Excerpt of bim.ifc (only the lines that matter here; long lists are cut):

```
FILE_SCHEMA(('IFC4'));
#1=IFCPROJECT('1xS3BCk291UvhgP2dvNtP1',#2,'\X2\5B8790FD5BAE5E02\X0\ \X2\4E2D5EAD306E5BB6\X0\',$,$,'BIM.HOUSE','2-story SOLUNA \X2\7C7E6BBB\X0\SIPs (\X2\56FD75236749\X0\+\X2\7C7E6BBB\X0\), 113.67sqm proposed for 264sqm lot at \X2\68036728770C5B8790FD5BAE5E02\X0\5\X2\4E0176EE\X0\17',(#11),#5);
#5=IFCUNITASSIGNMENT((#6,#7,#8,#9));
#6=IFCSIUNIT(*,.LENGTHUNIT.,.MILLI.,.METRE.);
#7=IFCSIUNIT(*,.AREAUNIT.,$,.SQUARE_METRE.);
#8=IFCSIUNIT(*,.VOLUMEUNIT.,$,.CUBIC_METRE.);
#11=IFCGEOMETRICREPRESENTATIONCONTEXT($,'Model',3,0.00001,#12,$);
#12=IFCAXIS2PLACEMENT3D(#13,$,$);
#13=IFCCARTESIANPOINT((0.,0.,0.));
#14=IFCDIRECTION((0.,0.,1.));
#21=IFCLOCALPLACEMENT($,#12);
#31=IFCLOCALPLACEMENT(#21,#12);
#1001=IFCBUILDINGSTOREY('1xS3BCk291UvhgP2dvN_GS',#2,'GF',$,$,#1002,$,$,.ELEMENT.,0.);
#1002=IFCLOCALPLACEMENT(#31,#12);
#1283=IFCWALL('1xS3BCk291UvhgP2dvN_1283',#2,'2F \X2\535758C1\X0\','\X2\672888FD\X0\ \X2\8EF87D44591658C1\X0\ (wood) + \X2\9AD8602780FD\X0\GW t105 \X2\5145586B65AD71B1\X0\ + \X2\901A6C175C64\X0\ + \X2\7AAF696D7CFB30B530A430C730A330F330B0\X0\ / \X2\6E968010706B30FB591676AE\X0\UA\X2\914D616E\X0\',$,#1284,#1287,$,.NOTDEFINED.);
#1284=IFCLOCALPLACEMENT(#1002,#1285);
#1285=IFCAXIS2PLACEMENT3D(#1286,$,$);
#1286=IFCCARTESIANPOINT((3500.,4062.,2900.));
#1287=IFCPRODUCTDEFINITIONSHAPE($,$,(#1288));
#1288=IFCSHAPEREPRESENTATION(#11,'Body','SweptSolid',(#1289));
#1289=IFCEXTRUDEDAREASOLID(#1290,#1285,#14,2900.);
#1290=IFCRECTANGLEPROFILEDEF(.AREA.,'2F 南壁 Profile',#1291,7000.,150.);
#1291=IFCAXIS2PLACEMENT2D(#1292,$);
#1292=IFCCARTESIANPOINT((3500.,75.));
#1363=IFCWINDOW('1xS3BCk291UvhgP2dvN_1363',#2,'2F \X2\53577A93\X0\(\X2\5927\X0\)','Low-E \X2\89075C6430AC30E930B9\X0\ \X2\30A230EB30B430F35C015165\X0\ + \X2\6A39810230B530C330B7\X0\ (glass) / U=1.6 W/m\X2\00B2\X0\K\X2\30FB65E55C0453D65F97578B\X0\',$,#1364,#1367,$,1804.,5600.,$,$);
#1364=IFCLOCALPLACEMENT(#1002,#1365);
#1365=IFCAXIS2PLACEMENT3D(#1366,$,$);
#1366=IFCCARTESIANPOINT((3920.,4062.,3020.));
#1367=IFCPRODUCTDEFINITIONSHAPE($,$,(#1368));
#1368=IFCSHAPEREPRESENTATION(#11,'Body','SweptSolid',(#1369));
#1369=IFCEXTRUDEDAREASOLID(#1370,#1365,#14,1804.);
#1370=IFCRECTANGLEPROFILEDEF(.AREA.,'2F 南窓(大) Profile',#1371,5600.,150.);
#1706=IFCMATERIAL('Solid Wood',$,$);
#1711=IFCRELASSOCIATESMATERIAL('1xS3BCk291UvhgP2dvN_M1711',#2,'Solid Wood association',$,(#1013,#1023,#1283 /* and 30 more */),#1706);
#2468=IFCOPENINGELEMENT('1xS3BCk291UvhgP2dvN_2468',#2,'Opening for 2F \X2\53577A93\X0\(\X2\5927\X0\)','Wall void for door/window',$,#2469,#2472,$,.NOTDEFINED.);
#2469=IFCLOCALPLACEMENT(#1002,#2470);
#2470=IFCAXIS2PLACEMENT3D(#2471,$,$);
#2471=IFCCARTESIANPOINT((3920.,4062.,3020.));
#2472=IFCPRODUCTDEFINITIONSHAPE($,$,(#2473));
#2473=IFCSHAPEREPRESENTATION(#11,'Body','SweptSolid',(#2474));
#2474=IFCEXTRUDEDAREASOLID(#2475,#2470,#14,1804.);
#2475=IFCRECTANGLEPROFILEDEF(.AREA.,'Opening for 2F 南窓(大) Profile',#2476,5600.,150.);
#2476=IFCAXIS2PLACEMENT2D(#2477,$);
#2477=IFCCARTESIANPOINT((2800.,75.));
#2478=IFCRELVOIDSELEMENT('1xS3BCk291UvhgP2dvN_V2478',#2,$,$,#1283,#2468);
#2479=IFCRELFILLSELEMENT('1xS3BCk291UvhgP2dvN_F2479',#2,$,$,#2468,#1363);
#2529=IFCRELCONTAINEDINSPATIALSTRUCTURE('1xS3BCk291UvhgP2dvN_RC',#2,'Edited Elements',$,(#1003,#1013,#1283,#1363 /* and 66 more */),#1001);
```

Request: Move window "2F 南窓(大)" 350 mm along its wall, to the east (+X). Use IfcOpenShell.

```python
import ifcopenshell
import ifcopenshell.api.geometry
import ifcopenshell.util.placement
import ifcopenshell.util.unit

model = ifcopenshell.open("bim.ifc")
unit_scale = ifcopenshell.util.unit.calculate_unit_scale(model)

window = model.by_guid("1xS3BCk291UvhgP2dvN_1363")
opening = window.FillsVoids[0].RelatingOpeningElement
wall = opening.VoidsElements[0].RelatingBuildingElement

wall_matrix = ifcopenshell.util.placement.get_local_placement(wall.ObjectPlacement)
shift = wall_matrix[:3, 0] * 0.35 / unit_scale
before = ifcopenshell.util.placement.get_local_placement(window.ObjectPlacement)[:3, 3].copy()

# The window is not placed relative to its opening, so move both.
for product in (opening, window):
    matrix = ifcopenshell.util.placement.get_local_placement(product.ObjectPlacement)
    matrix[:3, 3] += shift
    ifcopenshell.api.geometry.edit_object_placement(model, product=product, matrix=matrix, is_si=False)

after = ifcopenshell.util.placement.get_local_placement(window.ObjectPlacement)[:3, 3]
print("window moved by", (after - before).round(3) + 0.0)

model.write("bim_rev.ifc")
```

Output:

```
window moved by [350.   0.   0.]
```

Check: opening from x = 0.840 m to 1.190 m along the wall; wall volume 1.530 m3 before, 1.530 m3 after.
